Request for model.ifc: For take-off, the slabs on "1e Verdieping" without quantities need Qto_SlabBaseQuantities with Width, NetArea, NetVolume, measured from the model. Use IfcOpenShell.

First a look at what the model holds.

```python
import ifcopenshell
import ifcopenshell.util.element
import ifcopenshell.util.unit

model = ifcopenshell.open("model.ifc")
print(model.schema)
for unit_type in ("LENGTHUNIT", "AREAUNIT", "VOLUMEUNIT"):
    print(unit_type, ifcopenshell.util.unit.calculate_unit_scale(model, unit_type))
storey = next(s for s in model.by_type("IfcBuildingStorey") if s.Name == "1e Verdieping")
slabs = [e for e in ifcopenshell.util.element.get_decomposition(storey) if e.is_a("IfcSlab")]
for e in sorted(slabs, key=lambda e: e.id()):
    print(e.id(), e.is_a(), e.Name, list(ifcopenshell.util.element.get_psets(e, qtos_only=True)), sep=" | ")
```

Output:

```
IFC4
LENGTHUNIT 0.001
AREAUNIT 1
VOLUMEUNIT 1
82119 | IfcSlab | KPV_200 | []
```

```python
import ifcopenshell
import ifcopenshell.api.pset
import ifcopenshell.geom
import ifcopenshell.util.element
import ifcopenshell.util.shape
import ifcopenshell.util.unit

model = ifcopenshell.open("model.ifc")
unit_scale = ifcopenshell.util.unit.calculate_unit_scale(model)
area_scale = ifcopenshell.util.unit.calculate_unit_scale(model, "AREAUNIT")
volume_scale = ifcopenshell.util.unit.calculate_unit_scale(model, "VOLUMEUNIT")
settings = ifcopenshell.geom.settings()

storey = next(s for s in model.by_type("IfcBuildingStorey") if s.Name == "1e Verdieping")
slabs = [e for e in ifcopenshell.util.element.get_decomposition(storey) if e.is_a("IfcSlab")]

for e in sorted(slabs, key=lambda e: e.id()):
    if ifcopenshell.util.element.get_psets(e, qtos_only=True, should_inherit=False):
        continue
    # Geometry comes back in metres, in the element's own axes.
    shape = ifcopenshell.geom.create_shape(settings, e)
    values = {
        "Width": ifcopenshell.util.shape.get_z(shape.geometry) / unit_scale,
        "NetArea": ifcopenshell.util.shape.get_footprint_area(shape.geometry) / area_scale,
        "NetVolume": ifcopenshell.util.shape.get_volume(shape.geometry) / volume_scale,
    }
    qto = ifcopenshell.api.pset.add_qto(model, product=e, name="Qto_SlabBaseQuantities")
    ifcopenshell.api.pset.edit_qto(model, qto=qto, properties=values)
    print(e.id(), {k: round(v, 3) for k, v in values.items()})

model.write("model_edited.ifc")
```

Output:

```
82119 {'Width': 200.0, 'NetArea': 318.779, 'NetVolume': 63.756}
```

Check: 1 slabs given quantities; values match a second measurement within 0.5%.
